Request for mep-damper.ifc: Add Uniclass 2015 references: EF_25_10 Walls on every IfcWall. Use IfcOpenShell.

First a look at what the model holds.

```python
import ifcopenshell

model = ifcopenshell.open("mep-damper.ifc")
print(model.schema)
print("classifications:", [c.Name for c in model.by_type("IfcClassification")])
for ifc_class in ("IfcDoor", "IfcRoof", "IfcStair", "IfcWall", "IfcWindow"):
    print(ifc_class, len(model.by_type(ifc_class)))
```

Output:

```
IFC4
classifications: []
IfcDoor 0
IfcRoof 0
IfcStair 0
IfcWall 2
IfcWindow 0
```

```python
import ifcopenshell
import ifcopenshell.api.classification

model = ifcopenshell.open("mep-damper.ifc")

system = ifcopenshell.api.classification.add_classification(model, classification="Uniclass 2015")

codes = {
    "IfcWall": ("EF_25_10", "Walls"),
}
for ifc_class, (code, name) in codes.items():
    products = model.by_type(ifc_class)
    ifcopenshell.api.classification.add_reference(
        model, products=products, classification=system, identification=code, name=name
    )
    print(code, len(products))

model.write("mep-damper-out.ifc")
```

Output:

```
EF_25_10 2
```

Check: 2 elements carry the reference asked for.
